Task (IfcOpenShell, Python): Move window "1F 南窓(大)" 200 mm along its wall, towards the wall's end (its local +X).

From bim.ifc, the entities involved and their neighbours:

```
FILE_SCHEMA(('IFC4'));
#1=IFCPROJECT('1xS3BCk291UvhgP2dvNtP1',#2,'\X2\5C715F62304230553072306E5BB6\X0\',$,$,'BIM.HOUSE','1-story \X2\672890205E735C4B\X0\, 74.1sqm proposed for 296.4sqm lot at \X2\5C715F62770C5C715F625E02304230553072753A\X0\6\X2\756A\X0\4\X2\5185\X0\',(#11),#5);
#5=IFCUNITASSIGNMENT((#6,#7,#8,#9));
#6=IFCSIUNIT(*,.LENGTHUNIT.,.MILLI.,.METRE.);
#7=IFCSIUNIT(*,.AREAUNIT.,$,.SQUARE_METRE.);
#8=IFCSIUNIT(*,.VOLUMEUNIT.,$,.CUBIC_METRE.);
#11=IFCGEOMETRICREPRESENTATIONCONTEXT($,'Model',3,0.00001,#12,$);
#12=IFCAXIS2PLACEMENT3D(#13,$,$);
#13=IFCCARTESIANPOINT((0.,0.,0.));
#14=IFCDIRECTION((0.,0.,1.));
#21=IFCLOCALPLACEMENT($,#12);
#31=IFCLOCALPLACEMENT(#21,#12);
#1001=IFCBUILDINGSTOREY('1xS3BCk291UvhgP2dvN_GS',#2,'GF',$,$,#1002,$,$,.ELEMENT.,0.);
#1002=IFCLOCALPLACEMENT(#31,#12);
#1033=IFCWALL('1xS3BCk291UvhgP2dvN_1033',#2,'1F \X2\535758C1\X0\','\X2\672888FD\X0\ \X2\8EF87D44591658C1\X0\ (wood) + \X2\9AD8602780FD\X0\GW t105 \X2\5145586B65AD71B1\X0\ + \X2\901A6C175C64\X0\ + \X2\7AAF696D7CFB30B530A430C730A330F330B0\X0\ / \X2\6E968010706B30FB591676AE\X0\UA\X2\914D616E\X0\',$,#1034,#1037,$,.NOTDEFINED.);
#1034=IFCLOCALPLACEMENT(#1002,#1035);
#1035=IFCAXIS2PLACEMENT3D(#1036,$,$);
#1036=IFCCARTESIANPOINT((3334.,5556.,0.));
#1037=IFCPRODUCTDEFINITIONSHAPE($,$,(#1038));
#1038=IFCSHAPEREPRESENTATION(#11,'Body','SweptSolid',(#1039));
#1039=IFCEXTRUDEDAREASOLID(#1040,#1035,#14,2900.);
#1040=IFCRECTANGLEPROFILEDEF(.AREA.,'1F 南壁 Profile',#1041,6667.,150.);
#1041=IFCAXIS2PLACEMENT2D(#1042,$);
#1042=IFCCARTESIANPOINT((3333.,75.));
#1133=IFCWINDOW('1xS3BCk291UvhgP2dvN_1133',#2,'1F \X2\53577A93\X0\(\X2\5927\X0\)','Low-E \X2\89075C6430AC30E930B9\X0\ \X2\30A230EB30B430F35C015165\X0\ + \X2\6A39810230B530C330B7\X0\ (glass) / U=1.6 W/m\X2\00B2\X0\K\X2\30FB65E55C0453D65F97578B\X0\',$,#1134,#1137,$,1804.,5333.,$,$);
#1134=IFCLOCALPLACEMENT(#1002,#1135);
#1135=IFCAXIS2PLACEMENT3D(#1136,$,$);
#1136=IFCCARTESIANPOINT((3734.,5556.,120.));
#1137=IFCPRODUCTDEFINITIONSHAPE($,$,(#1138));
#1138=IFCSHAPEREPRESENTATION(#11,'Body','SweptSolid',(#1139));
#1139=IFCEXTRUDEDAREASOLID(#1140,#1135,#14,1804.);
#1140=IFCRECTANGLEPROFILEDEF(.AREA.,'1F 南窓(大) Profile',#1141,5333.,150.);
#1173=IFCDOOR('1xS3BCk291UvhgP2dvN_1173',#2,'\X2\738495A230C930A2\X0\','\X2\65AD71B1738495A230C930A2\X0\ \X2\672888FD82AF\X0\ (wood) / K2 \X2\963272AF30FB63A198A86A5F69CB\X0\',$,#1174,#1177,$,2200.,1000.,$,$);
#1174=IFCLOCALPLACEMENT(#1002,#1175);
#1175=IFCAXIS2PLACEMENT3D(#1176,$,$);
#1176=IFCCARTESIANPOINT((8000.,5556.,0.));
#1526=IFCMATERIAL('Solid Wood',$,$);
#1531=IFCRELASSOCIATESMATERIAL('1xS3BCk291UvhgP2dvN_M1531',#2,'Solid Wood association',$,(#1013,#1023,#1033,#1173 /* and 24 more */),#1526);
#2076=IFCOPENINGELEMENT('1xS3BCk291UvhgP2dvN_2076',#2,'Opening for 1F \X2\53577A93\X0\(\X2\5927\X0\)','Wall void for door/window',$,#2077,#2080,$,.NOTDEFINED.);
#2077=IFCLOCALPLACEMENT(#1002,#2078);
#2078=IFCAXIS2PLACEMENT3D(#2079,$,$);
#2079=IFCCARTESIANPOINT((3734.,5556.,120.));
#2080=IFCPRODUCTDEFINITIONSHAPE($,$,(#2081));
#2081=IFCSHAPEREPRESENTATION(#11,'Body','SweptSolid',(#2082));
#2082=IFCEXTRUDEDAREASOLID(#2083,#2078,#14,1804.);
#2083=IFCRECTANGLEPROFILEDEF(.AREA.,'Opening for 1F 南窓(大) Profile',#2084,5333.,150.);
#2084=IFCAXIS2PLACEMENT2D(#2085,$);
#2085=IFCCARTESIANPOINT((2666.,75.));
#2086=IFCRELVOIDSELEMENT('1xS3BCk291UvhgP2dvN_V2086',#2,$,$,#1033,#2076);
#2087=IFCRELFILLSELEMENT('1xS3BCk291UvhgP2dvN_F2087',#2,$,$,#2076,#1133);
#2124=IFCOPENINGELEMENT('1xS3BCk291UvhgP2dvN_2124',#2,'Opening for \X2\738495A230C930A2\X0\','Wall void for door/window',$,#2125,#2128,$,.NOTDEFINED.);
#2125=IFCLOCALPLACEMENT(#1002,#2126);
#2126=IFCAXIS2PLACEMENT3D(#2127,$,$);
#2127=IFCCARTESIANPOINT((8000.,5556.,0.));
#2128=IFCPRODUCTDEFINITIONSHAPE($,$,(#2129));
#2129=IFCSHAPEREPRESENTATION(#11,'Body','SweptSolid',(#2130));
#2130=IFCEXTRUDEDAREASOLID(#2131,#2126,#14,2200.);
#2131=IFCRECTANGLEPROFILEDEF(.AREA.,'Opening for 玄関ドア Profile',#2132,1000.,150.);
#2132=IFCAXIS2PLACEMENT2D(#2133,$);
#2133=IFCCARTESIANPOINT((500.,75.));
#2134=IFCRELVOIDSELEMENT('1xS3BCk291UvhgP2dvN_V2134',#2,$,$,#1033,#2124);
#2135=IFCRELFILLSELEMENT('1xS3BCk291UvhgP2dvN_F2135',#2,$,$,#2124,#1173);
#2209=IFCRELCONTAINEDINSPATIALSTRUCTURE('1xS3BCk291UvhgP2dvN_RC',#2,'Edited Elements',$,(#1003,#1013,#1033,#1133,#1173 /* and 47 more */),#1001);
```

```python
import ifcopenshell
import ifcopenshell.api.geometry
import ifcopenshell.util.placement
import ifcopenshell.util.unit

model = ifcopenshell.open("bim.ifc")
unit_scale = ifcopenshell.util.unit.calculate_unit_scale(model)

window = model.by_guid("1xS3BCk291UvhgP2dvN_1133")
opening = window.FillsVoids[0].RelatingOpeningElement
wall = opening.VoidsElements[0].RelatingBuildingElement

wall_matrix = ifcopenshell.util.placement.get_local_placement(wall.ObjectPlacement)
shift = wall_matrix[:3, 0] * 0.2 / unit_scale
before = ifcopenshell.util.placement.get_local_placement(window.ObjectPlacement)[:3, 3].copy()

# The window is not placed relative to its opening, so move both.
for product in (opening, window):
    matrix = ifcopenshell.util.placement.get_local_placement(product.ObjectPlacement)
    matrix[:3, 3] += shift
    ifcopenshell.api.geometry.edit_object_placement(model, product=product, matrix=matrix, is_si=False)

after = ifcopenshell.util.placement.get_local_placement(window.ObjectPlacement)[:3, 3]
print("window moved by", (after - before).round(3) + 0.0)

model.write("bim_edited.ifc")
```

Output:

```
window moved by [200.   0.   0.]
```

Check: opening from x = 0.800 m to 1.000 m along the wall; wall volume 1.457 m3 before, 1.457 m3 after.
